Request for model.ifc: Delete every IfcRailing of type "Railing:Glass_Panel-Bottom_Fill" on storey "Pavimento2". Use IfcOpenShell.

First a look at what the model holds.

```python
import ifcopenshell
import ifcopenshell.util.element

model = ifcopenshell.open("model.ifc")
print(model.schema)
storey = next(s for s in model.by_type("IfcBuildingStorey") if s.Name == "Pavimento2")
railings = [e for e in ifcopenshell.util.element.get_decomposition(storey) if e.is_a("IfcRailing")]
seen = {}
for e in railings:
    element_type = ifcopenshell.util.element.get_type(e)
    name = element_type.Name if element_type not in (None, e) else None
    seen[name] = seen.get(name, 0) + 1
for name, count in sorted(seen.items(), key=str):
    print(count, "x", name)
```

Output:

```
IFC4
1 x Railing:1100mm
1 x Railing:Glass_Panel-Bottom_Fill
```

```python
import ifcopenshell
import ifcopenshell.api.root
import ifcopenshell.util.element

model = ifcopenshell.open("model.ifc")

storey = next(s for s in model.by_type("IfcBuildingStorey") if s.Name == "Pavimento2")
railings = [e for e in ifcopenshell.util.element.get_decomposition(storey) if e.is_a("IfcRailing")]
targets = [e for e in railings if (t := ifcopenshell.util.element.get_type(e)) not in (None, e) and t.Name == "Railing:Glass_Panel-Bottom_Fill"]

for e in targets:
    ifcopenshell.api.root.remove_product(model, product=e)
print(len(targets), "removed")

model.write("model_rev.ifc")
```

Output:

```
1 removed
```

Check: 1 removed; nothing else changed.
